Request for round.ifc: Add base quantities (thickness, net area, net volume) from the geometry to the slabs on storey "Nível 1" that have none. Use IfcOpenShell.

First a look at what the model holds.

```python
import ifcopenshell
import ifcopenshell.util.element
import ifcopenshell.util.unit

model = ifcopenshell.open("round.ifc")
print(model.schema)
for unit_type in ("LENGTHUNIT", "AREAUNIT", "VOLUMEUNIT"):
    print(unit_type, ifcopenshell.util.unit.calculate_unit_scale(model, unit_type))
storey = next(s for s in model.by_type("IfcBuildingStorey") if s.Name == "Nível 1")
slabs = [e for e in ifcopenshell.util.element.get_decomposition(storey) if e.is_a("IfcSlab")]
for e in sorted(slabs, key=lambda e: e.id()):
    print(e.id(), e.is_a(), e.Name, list(ifcopenshell.util.element.get_psets(e, qtos_only=True)), sep=" | ")
```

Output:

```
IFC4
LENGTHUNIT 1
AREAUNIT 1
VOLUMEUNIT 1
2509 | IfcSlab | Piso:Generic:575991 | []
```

```python
import ifcopenshell
import ifcopenshell.api.pset
import ifcopenshell.geom
import ifcopenshell.util.element
import ifcopenshell.util.shape
import ifcopenshell.util.unit

model = ifcopenshell.open("round.ifc")
unit_scale = ifcopenshell.util.unit.calculate_unit_scale(model)
area_scale = ifcopenshell.util.unit.calculate_unit_scale(model, "AREAUNIT")
volume_scale = ifcopenshell.util.unit.calculate_unit_scale(model, "VOLUMEUNIT")
settings = ifcopenshell.geom.settings()

storey = next(s for s in model.by_type("IfcBuildingStorey") if s.Name == "Nível 1")
slabs = [e for e in ifcopenshell.util.element.get_decomposition(storey) if e.is_a("IfcSlab")]

for e in sorted(slabs, key=lambda e: e.id()):
    if ifcopenshell.util.element.get_psets(e, qtos_only=True, should_inherit=False):
        continue
    # Geometry comes back in metres, in the element's own axes.
    shape = ifcopenshell.geom.create_shape(settings, e)
    values = {
        "Width": ifcopenshell.util.shape.get_z(shape.geometry) / unit_scale,
        "NetArea": ifcopenshell.util.shape.get_footprint_area(shape.geometry) / area_scale,
        "NetVolume": ifcopenshell.util.shape.get_volume(shape.geometry) / volume_scale,
    }
    qto = ifcopenshell.api.pset.add_qto(model, product=e, name="Qto_SlabBaseQuantities")
    ifcopenshell.api.pset.edit_qto(model, qto=qto, properties=values)
    print(e.id(), {k: round(v, 3) for k, v in values.items()})

model.write("round_edited.ifc")
```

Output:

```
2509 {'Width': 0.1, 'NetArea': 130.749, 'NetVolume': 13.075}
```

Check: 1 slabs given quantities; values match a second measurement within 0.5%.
